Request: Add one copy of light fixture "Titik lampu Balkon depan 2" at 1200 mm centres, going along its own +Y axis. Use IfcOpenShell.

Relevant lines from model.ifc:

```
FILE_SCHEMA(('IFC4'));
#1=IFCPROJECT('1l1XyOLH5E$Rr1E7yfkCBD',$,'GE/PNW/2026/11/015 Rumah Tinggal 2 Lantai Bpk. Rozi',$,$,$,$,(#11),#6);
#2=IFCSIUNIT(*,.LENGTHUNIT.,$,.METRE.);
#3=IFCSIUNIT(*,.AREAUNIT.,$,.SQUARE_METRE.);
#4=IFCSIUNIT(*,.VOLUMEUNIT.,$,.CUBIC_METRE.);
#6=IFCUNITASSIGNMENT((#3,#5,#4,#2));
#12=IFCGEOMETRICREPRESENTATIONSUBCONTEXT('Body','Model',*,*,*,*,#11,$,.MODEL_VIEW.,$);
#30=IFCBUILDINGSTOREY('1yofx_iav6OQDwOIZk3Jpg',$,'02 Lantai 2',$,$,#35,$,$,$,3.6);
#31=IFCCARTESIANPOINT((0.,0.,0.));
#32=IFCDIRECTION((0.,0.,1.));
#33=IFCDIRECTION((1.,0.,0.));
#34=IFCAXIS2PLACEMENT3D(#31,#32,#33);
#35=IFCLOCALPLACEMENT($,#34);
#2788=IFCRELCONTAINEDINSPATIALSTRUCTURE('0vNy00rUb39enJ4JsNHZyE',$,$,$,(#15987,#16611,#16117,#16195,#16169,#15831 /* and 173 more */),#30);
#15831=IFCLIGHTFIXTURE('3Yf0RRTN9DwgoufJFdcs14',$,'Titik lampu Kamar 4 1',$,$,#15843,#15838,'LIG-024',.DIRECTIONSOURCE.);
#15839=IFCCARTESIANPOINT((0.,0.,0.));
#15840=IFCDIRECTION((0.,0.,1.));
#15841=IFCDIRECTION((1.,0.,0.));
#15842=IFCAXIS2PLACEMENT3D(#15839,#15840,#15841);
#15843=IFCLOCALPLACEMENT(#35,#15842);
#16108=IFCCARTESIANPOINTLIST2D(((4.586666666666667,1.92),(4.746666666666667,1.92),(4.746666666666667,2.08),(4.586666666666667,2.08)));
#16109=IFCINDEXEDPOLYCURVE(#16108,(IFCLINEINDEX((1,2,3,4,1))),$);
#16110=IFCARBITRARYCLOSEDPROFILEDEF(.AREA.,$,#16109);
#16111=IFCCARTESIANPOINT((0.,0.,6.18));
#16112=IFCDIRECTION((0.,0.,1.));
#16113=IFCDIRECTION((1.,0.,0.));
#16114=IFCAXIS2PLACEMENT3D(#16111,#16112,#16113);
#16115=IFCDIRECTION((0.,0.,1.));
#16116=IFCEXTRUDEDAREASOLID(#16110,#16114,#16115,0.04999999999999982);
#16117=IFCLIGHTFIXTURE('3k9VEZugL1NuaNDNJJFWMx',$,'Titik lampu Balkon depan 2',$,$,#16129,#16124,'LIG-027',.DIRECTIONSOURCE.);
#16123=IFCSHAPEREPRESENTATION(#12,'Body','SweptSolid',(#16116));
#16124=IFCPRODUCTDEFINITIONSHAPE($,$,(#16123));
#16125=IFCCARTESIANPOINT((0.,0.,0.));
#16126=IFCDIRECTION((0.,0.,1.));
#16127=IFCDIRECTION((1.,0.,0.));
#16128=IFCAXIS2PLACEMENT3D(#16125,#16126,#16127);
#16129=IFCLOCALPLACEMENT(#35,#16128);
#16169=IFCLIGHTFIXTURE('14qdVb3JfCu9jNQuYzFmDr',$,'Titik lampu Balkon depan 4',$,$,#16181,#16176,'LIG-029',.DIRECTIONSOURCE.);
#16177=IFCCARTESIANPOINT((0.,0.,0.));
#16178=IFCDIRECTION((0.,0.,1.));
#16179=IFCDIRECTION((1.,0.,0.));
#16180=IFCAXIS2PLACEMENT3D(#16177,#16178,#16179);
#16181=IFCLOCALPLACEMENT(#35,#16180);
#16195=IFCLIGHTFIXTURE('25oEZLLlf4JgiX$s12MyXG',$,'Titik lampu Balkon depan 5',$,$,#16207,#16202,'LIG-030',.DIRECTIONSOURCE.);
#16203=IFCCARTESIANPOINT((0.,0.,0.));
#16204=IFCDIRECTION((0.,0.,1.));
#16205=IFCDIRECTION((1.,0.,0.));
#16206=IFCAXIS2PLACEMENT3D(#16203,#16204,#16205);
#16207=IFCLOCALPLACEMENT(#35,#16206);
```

```python
import ifcopenshell
import ifcopenshell.api.geometry
import ifcopenshell.api.root
import ifcopenshell.util.element
import ifcopenshell.util.placement
import ifcopenshell.util.unit

model = ifcopenshell.open("model.ifc")
unit_scale = ifcopenshell.util.unit.calculate_unit_scale(model)

source = model.by_guid("3k9VEZugL1NuaNDNJJFWMx")
base = ifcopenshell.util.placement.get_local_placement(source.ObjectPlacement)
step = base[:3, 1] * 1.2 / unit_scale

for i in range(1, 2):
    copy = ifcopenshell.api.root.copy_class(model, product=source)
    copy.Representation = ifcopenshell.util.element.copy_deep(
        model, source.Representation, exclude=["IfcGeometricRepresentationContext", "IfcRepresentationMap"]
    )
    copy.Tag = None
    matrix = base.copy()
    matrix[:3, 3] += i * step
    print("added at", matrix[:3, 3].round(3) + 0.0)
    ifcopenshell.api.geometry.edit_object_placement(model, product=copy, matrix=matrix, is_si=False)

model.write("model_edited.ifc")
```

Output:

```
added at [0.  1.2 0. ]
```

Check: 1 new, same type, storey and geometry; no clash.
